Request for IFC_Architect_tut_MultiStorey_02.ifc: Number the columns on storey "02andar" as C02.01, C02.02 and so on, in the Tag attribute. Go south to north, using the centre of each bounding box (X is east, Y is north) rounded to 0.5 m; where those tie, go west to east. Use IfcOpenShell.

First a look at what the model holds.

```python
import ifcopenshell
import ifcopenshell.util.element
import ifcopenshell.util.placement

model = ifcopenshell.open("IFC_Architect_tut_MultiStorey_02.ifc")
print(model.schema)
storey = next(s for s in model.by_type("IfcBuildingStorey") if s.Name == "02andar")
columns = [e for e in ifcopenshell.util.element.get_decomposition(storey) if e.is_a("IfcColumn")]
for e in sorted(columns, key=lambda e: e.id()):
    origin = ifcopenshell.util.placement.get_local_placement(e.ObjectPlacement)[:3, 3]
    print(e.id(), e.Tag, e.Name, origin.round(2) + 0.0, sep=" | ")
```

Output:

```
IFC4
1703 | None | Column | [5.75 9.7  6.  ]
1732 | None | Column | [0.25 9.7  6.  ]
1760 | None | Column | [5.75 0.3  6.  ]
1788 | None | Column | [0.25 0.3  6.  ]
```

```python
import ifcopenshell
import ifcopenshell.geom
import ifcopenshell.util.element
import ifcopenshell.util.shape

model = ifcopenshell.open("IFC_Architect_tut_MultiStorey_02.ifc")
settings = ifcopenshell.geom.settings()
settings.set("use-world-coords", True)


def centre(element):
    shape = ifcopenshell.geom.create_shape(settings, element)
    return ifcopenshell.util.shape.get_bbox_centroid(shape.geometry)


storey = next(s for s in model.by_type("IfcBuildingStorey") if s.Name == "02andar")
columns = [e for e in ifcopenshell.util.element.get_decomposition(storey) if e.is_a("IfcColumn")]

# Insertion points can sit at a corner or the storey origin, so sort by the geometry (in metres).
centres = {e: centre(e) for e in columns}
columns.sort(key=lambda e: (round(centres[e][1] / 0.5), centres[e][0]))

for i, e in enumerate(columns, start=1):
    number = f"C02.{i:02d}"
    e.Tag = number
    print(e.id(), number)

model.write("IFC_Architect_tut_MultiStorey_02_rev.ifc")
```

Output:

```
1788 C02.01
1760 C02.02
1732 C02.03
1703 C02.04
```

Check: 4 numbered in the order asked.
